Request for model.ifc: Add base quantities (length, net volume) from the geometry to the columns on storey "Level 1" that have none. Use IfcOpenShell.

First a look at what the model holds.

```python
import ifcopenshell
import ifcopenshell.util.element
import ifcopenshell.util.unit

model = ifcopenshell.open("model.ifc")
print(model.schema)
for unit_type in ("LENGTHUNIT", "AREAUNIT", "VOLUMEUNIT"):
    print(unit_type, ifcopenshell.util.unit.calculate_unit_scale(model, unit_type))
storey = next(s for s in model.by_type("IfcBuildingStorey") if s.Name == "Level 1")
columns = [e for e in ifcopenshell.util.element.get_decomposition(storey) if e.is_a("IfcColumn")]
for e in sorted(columns, key=lambda e: e.id()):
    print(e.id(), e.is_a(), e.Name, list(ifcopenshell.util.element.get_psets(e, qtos_only=True)), sep=" | ")
```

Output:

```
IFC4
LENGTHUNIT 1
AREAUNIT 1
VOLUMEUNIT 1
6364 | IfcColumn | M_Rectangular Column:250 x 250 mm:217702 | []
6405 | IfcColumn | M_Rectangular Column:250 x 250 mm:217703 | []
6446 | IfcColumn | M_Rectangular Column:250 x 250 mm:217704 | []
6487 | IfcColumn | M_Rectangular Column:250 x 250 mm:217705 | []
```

```python
import ifcopenshell
import ifcopenshell.api.pset
import ifcopenshell.geom
import ifcopenshell.util.element
import ifcopenshell.util.shape
import ifcopenshell.util.unit

model = ifcopenshell.open("model.ifc")
unit_scale = ifcopenshell.util.unit.calculate_unit_scale(model)
volume_scale = ifcopenshell.util.unit.calculate_unit_scale(model, "VOLUMEUNIT")
settings = ifcopenshell.geom.settings()

storey = next(s for s in model.by_type("IfcBuildingStorey") if s.Name == "Level 1")
columns = [e for e in ifcopenshell.util.element.get_decomposition(storey) if e.is_a("IfcColumn")]

for e in sorted(columns, key=lambda e: e.id()):
    if ifcopenshell.util.element.get_psets(e, qtos_only=True, should_inherit=False):
        continue
    # Geometry comes back in metres, in the element's own axes.
    shape = ifcopenshell.geom.create_shape(settings, e)
    values = {
        "Length": ifcopenshell.util.shape.get_z(shape.geometry) / unit_scale,
        "NetVolume": ifcopenshell.util.shape.get_volume(shape.geometry) / volume_scale,
    }
    qto = ifcopenshell.api.pset.add_qto(model, product=e, name="Qto_ColumnBaseQuantities")
    ifcopenshell.api.pset.edit_qto(model, qto=qto, properties=values)
    print(e.id(), {k: round(v, 3) for k, v in values.items()})

model.write("model_rev.ifc")
```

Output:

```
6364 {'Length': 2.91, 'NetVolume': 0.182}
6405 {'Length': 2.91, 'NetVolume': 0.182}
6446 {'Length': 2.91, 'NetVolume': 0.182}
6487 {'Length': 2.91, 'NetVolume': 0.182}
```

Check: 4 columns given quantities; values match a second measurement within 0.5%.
